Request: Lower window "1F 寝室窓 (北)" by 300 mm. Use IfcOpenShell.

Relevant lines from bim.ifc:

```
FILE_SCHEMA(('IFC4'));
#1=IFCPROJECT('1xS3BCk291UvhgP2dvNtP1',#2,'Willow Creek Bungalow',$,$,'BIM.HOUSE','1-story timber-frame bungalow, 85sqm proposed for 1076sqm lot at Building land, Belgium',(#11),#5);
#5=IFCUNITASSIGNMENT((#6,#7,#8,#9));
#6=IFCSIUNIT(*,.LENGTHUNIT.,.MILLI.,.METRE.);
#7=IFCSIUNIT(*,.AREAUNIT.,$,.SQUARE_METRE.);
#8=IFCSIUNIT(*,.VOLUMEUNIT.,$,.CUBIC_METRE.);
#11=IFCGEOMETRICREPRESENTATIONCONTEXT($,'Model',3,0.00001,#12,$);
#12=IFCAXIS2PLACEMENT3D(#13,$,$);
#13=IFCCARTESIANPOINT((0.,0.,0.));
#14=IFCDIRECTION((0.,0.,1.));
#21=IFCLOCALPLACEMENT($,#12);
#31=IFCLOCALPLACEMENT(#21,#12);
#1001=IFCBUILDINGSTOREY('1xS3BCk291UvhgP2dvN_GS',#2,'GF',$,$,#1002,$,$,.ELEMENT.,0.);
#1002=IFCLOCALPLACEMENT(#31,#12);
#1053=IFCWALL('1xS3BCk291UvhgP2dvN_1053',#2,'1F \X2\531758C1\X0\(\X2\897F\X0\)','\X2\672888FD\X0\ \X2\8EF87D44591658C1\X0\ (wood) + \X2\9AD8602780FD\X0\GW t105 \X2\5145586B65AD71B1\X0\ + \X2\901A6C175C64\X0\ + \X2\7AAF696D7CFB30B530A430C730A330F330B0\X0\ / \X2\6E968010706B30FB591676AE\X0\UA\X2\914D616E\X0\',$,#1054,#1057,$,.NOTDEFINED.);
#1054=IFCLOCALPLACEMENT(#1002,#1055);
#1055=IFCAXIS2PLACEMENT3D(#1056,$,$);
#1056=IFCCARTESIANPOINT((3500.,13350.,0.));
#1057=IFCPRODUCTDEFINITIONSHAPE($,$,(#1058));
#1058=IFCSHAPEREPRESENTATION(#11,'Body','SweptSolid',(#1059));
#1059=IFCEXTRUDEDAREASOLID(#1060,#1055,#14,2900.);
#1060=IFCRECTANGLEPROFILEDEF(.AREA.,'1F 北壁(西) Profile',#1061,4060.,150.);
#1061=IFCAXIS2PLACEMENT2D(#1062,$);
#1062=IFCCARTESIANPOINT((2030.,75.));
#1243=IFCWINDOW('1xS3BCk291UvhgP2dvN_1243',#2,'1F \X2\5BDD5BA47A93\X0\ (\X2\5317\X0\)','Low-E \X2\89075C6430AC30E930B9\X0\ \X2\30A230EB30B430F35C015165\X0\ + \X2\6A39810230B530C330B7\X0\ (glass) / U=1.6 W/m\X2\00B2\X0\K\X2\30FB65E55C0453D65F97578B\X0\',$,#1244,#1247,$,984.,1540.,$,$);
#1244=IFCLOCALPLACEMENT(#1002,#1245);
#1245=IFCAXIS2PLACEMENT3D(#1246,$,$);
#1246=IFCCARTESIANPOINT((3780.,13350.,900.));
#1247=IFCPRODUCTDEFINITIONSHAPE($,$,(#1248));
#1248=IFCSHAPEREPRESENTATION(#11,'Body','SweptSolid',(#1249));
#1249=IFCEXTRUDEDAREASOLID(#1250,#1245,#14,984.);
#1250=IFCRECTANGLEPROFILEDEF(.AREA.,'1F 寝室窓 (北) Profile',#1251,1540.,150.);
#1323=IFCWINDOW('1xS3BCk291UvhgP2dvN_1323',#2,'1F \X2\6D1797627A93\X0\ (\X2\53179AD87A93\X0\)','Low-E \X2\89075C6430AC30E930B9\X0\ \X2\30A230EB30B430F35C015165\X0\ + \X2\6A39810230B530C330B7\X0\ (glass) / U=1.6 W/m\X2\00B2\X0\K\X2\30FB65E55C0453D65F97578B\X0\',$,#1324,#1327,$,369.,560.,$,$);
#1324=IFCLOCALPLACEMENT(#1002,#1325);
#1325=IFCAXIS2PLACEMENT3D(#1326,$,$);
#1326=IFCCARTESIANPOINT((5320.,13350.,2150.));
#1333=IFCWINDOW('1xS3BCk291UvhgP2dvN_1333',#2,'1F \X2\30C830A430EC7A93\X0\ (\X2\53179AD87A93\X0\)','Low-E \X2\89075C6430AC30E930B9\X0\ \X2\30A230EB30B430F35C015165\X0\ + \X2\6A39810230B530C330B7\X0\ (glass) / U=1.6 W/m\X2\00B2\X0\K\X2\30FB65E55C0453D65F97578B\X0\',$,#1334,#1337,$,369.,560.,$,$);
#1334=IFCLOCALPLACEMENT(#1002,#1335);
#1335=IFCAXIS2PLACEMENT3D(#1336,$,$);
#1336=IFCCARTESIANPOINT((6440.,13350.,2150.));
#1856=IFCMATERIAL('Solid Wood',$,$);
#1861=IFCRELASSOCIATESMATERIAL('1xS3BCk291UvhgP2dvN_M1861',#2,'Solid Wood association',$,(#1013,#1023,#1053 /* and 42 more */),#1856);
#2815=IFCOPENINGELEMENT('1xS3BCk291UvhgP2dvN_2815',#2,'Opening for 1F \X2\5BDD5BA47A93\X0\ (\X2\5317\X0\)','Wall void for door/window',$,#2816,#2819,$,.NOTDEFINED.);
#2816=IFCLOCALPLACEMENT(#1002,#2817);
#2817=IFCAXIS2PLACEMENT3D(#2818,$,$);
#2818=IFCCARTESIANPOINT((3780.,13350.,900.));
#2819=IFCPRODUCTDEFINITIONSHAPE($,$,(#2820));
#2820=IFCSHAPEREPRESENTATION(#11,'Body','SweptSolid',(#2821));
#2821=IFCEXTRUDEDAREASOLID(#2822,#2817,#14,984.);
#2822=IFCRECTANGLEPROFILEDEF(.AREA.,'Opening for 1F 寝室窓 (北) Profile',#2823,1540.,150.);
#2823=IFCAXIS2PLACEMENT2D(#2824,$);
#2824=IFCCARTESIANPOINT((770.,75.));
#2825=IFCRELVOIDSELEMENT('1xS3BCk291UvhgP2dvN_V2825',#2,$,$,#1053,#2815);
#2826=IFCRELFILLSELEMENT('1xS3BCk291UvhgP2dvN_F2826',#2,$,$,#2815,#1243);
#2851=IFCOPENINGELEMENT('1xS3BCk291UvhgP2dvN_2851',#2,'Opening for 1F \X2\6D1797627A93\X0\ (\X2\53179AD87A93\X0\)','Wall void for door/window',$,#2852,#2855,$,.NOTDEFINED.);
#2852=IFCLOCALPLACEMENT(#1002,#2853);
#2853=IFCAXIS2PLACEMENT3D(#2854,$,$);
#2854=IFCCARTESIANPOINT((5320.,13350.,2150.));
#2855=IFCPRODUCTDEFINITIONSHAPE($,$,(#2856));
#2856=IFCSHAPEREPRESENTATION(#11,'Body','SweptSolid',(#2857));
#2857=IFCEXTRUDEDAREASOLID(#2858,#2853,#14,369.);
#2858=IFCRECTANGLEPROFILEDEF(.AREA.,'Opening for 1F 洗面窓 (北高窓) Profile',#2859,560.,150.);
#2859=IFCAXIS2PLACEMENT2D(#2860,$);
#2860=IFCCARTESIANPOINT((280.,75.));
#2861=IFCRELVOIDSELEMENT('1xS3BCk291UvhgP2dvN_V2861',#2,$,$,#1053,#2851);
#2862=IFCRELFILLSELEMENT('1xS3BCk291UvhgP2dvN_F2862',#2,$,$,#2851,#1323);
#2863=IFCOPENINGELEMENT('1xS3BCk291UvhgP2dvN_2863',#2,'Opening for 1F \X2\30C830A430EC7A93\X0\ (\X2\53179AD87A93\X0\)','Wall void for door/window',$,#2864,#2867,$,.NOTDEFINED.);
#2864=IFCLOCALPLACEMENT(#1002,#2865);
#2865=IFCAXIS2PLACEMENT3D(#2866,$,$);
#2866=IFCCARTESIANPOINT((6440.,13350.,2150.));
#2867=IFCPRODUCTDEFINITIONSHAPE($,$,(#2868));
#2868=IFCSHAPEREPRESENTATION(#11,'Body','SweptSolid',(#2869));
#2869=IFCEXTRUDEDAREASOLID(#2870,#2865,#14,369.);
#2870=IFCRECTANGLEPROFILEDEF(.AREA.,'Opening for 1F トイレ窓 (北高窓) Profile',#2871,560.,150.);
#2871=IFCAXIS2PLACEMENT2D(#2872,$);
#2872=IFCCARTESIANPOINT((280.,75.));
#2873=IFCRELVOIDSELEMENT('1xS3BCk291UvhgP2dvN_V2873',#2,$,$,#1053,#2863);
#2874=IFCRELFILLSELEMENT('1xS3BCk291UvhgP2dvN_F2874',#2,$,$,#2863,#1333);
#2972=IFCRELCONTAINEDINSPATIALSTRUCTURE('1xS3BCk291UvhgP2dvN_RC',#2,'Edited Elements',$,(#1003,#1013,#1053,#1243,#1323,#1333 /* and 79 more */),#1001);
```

```python
import numpy as np
import ifcopenshell
import ifcopenshell.api.geometry
import ifcopenshell.util.placement
import ifcopenshell.util.unit

model = ifcopenshell.open("bim.ifc")
unit_scale = ifcopenshell.util.unit.calculate_unit_scale(model)

window = model.by_guid("1xS3BCk291UvhgP2dvN_1243")
opening = window.FillsVoids[0].RelatingOpeningElement
dz = -0.3 / unit_scale

shift = np.array([0.0, 0.0, dz])
# The window is not placed relative to its opening, so move both.
for product in (opening, window):
    matrix = ifcopenshell.util.placement.get_local_placement(product.ObjectPlacement)
    matrix[:3, 3] += shift
    ifcopenshell.api.geometry.edit_object_placement(model, product=product, matrix=matrix, is_si=False)

print(f"moved by {dz * unit_scale:+.3f} m")

model.write("bim_rev.ifc")
```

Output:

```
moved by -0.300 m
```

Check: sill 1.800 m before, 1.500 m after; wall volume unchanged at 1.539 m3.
